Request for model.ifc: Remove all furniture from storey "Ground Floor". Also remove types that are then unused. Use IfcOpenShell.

First a look at what the model holds.

```python
import ifcopenshell
import ifcopenshell.util.element

model = ifcopenshell.open("model.ifc")
print(model.schema)
storey = next(s for s in model.by_type("IfcBuildingStorey") if s.Name == "Ground Floor")
furniture = [e for e in ifcopenshell.util.element.get_decomposition(storey) if e.is_a("IfcFurnishingElement")]
seen = {}
for e in furniture:
    element_type = ifcopenshell.util.element.get_type(e)
    name = element_type.Name if element_type not in (None, e) else None
    seen[name] = seen.get(name, 0) + 1
for name, count in sorted(seen.items(), key=str):
    print(count, "x", name)
```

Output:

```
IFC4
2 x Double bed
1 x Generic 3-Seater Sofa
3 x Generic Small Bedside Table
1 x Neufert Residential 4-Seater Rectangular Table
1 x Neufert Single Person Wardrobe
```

```python
import ifcopenshell
import ifcopenshell.api.root
import ifcopenshell.util.element

model = ifcopenshell.open("model.ifc")

storey = next(s for s in model.by_type("IfcBuildingStorey") if s.Name == "Ground Floor")
furniture = [e for e in ifcopenshell.util.element.get_decomposition(storey) if e.is_a("IfcFurnishingElement")]
types = {ifcopenshell.util.element.get_type(e) for e in furniture} - {None, *furniture}

for e in furniture:
    ifcopenshell.api.root.remove_product(model, product=e)
print(len(furniture), "removed")

unused = [t for t in types if not ifcopenshell.util.element.get_types(t)]
for t in unused:
    ifcopenshell.api.root.remove_product(model, product=t)
print(len(unused), "unused types removed")

model.write("model_rev.ifc")
```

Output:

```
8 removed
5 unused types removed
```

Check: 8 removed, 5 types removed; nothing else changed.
